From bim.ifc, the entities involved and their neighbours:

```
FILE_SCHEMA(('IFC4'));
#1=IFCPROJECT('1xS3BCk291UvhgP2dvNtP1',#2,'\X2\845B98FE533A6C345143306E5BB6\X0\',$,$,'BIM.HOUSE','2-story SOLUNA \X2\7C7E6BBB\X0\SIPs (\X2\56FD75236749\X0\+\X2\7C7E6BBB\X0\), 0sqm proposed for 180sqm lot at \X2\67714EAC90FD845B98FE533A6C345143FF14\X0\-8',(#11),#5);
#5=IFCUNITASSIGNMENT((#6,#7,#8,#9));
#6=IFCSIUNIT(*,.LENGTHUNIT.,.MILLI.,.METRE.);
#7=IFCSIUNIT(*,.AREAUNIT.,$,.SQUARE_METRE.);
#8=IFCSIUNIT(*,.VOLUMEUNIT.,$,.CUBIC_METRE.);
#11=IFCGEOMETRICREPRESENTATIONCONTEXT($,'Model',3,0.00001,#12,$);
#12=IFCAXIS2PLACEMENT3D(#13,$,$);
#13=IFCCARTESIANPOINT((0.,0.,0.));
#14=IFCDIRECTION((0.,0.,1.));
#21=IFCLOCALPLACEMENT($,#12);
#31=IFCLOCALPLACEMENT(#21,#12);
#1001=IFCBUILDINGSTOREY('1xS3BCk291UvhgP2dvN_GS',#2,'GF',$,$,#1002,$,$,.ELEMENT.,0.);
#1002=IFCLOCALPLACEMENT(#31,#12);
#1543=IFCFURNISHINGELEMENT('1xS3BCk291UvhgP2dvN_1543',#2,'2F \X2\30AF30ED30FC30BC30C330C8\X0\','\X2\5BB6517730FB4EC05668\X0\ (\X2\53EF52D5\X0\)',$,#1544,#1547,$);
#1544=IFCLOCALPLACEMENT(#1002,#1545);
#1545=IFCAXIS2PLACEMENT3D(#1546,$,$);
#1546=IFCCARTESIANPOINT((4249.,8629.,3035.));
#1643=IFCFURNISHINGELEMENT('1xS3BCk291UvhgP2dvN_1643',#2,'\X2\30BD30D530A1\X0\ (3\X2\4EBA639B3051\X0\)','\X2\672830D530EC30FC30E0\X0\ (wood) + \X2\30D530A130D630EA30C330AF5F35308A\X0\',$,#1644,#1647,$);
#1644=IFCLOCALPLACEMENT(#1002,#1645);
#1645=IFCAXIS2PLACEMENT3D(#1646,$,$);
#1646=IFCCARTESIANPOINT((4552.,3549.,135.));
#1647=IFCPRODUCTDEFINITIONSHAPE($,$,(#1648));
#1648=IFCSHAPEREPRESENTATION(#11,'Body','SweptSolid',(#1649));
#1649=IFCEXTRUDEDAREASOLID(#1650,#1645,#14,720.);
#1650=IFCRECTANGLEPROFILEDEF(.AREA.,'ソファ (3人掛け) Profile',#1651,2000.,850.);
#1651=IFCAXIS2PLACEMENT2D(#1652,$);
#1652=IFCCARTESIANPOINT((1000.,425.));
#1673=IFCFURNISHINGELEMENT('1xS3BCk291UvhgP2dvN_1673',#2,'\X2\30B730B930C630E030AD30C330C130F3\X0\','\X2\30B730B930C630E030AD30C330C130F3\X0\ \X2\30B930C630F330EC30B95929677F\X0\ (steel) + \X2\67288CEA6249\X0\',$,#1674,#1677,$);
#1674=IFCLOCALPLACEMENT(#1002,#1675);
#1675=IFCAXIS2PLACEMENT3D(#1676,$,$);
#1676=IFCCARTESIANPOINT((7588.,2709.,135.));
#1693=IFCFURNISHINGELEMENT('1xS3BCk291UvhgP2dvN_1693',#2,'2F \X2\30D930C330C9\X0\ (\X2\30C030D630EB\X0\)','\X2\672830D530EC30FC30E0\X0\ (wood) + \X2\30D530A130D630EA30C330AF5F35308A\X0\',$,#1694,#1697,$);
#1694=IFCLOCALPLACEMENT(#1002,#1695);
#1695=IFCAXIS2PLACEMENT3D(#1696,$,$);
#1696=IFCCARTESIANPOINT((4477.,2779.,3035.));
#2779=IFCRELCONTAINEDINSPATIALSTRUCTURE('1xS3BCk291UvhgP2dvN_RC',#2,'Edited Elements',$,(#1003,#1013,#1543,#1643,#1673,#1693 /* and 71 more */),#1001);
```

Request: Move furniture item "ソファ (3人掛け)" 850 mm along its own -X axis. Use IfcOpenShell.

```python
import ifcopenshell
import ifcopenshell.api.geometry
import ifcopenshell.util.placement
import ifcopenshell.util.unit

model = ifcopenshell.open("bim.ifc")
unit_scale = ifcopenshell.util.unit.calculate_unit_scale(model)

item = model.by_id(1643)
matrix = ifcopenshell.util.placement.get_local_placement(item.ObjectPlacement)
matrix[:3, 3] -= matrix[:3, 0] * 0.85 / unit_scale
ifcopenshell.api.geometry.edit_object_placement(model, product=item, matrix=matrix, is_si=False)

print(ifcopenshell.util.placement.get_local_placement(item.ObjectPlacement).round(3) + 0.0)

model.write("bim_edited.ifc")
```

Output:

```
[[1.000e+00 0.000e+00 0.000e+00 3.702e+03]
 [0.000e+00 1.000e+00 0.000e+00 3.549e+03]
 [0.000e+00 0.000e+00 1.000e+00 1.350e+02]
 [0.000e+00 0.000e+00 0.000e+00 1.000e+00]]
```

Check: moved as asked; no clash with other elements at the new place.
